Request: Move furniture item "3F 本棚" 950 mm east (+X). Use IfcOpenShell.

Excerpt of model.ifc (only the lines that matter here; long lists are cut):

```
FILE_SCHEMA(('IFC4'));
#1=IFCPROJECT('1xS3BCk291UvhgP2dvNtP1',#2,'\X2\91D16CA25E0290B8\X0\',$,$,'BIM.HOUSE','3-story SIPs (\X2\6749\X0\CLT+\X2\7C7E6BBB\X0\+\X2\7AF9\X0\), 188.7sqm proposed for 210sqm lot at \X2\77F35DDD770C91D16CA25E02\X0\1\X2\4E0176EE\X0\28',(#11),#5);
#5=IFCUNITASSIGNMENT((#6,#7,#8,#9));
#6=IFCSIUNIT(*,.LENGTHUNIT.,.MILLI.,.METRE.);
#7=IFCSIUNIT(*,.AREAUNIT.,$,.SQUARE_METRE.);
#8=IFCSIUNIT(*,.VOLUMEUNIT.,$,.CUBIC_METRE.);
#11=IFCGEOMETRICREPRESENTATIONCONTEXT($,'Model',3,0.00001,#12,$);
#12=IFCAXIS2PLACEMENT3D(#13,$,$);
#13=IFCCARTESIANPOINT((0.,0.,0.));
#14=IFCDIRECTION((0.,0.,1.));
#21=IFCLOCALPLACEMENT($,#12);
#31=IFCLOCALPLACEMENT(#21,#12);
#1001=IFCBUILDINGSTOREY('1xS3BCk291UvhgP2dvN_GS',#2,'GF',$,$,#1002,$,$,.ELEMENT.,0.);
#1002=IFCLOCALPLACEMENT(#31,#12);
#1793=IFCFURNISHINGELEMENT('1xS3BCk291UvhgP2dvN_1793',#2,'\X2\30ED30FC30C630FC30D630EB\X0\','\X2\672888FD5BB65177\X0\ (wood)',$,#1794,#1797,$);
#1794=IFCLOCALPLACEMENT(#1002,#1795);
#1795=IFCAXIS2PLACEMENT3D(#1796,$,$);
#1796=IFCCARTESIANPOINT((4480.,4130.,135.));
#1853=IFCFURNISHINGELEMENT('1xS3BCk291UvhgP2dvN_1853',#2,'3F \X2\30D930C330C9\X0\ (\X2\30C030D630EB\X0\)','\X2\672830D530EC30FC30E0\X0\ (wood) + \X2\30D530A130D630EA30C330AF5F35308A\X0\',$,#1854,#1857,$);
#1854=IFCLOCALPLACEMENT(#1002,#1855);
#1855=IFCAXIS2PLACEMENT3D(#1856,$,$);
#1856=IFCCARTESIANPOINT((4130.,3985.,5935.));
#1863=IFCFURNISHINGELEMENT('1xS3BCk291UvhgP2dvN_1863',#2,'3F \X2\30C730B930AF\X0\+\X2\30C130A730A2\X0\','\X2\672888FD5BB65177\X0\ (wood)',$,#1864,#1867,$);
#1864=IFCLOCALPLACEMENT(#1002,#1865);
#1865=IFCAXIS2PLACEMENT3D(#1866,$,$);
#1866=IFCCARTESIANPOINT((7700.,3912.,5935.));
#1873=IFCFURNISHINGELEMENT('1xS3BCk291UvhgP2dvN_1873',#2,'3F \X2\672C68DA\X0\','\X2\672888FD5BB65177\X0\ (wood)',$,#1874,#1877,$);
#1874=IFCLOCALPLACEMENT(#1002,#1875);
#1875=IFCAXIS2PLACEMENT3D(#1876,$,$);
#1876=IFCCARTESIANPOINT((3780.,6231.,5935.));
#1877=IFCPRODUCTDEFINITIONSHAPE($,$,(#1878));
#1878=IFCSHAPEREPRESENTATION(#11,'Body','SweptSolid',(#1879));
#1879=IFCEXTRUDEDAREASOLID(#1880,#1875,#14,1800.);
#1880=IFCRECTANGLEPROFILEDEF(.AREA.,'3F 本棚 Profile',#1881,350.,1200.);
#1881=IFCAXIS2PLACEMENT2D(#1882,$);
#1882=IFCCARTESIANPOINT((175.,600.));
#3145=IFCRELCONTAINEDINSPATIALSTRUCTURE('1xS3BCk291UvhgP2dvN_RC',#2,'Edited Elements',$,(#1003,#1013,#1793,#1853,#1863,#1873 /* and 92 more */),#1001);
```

```python
import ifcopenshell
import ifcopenshell.api.geometry
import ifcopenshell.util.placement
import ifcopenshell.util.unit

model = ifcopenshell.open("model.ifc")
unit_scale = ifcopenshell.util.unit.calculate_unit_scale(model)

item = model.by_guid("1xS3BCk291UvhgP2dvN_1873")
matrix = ifcopenshell.util.placement.get_local_placement(item.ObjectPlacement)
matrix[0, 3] += 0.95 / unit_scale
ifcopenshell.api.geometry.edit_object_placement(model, product=item, matrix=matrix, is_si=False)

print(ifcopenshell.util.placement.get_local_placement(item.ObjectPlacement).round(3) + 0.0)

model.write("model_rev.ifc")
```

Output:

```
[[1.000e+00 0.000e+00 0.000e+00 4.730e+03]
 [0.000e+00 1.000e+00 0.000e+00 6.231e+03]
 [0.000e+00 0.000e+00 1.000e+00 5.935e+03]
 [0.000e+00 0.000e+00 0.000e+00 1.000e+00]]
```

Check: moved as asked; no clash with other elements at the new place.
